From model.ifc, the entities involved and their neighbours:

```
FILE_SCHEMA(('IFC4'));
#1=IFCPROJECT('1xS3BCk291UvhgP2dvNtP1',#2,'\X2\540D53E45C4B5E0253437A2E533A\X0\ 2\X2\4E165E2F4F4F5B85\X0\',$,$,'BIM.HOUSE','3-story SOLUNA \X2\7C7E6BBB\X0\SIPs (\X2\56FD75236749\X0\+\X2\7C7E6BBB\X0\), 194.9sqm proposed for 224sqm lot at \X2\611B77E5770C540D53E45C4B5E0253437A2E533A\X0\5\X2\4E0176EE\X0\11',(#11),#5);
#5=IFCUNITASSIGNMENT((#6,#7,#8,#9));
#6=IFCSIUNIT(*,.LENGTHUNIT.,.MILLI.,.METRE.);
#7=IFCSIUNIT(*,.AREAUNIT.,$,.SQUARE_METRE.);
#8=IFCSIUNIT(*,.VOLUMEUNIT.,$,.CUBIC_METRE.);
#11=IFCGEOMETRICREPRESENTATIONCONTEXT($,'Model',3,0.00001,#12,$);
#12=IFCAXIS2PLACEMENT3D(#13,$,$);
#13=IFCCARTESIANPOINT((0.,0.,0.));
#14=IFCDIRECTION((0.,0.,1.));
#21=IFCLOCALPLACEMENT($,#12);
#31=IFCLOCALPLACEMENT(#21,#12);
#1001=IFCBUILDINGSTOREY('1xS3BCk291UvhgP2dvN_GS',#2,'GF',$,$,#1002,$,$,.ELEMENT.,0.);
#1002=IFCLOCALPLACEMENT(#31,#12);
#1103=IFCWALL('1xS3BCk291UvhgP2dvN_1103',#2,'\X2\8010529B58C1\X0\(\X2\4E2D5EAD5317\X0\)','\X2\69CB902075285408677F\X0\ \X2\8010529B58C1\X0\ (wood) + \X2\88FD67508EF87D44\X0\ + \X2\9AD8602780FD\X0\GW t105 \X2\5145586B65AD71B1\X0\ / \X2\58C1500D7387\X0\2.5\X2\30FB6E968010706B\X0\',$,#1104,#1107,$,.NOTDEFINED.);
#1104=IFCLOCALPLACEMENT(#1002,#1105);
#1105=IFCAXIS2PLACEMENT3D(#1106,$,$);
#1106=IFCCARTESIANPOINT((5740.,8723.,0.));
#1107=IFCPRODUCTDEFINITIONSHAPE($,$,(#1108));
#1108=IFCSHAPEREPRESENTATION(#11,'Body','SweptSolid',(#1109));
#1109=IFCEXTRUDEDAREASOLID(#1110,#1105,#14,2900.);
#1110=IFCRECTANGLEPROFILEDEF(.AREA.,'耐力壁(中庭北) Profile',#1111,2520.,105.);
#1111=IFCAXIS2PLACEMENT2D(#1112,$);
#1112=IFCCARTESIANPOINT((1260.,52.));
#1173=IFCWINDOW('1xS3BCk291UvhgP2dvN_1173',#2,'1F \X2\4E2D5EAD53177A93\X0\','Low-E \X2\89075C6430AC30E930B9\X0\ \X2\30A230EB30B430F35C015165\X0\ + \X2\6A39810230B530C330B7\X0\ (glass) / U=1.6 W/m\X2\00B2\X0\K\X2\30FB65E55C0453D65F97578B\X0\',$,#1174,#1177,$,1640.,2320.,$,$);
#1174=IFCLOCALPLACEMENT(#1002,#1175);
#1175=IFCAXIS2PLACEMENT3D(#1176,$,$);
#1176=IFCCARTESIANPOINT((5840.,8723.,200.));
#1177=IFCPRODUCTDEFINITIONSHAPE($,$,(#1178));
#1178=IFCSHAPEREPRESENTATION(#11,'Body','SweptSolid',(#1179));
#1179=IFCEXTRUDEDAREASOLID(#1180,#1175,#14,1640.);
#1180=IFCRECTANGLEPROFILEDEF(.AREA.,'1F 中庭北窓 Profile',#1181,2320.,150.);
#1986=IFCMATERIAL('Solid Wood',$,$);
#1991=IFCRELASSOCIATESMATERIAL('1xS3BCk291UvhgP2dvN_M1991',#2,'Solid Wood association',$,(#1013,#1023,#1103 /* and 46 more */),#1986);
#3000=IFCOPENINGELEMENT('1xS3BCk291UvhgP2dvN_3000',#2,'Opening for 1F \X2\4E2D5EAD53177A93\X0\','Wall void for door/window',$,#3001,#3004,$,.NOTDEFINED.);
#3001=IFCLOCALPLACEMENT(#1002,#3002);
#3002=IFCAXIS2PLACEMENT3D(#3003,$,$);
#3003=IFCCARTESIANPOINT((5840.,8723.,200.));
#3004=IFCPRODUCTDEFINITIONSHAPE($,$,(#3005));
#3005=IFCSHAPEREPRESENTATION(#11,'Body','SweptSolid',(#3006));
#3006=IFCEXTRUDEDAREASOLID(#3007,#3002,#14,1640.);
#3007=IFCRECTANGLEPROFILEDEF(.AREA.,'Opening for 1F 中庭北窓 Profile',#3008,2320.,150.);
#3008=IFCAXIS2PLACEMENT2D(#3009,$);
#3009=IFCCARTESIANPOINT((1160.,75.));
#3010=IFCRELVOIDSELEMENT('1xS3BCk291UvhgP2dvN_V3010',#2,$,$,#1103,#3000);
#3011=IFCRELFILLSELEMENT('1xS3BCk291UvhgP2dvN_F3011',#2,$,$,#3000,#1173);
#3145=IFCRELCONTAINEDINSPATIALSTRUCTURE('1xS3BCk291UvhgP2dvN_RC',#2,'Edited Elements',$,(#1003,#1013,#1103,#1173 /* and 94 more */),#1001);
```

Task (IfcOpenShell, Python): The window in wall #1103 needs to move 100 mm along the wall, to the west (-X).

```python
import ifcopenshell
import ifcopenshell.api.geometry
import ifcopenshell.util.placement
import ifcopenshell.util.unit

model = ifcopenshell.open("model.ifc")
unit_scale = ifcopenshell.util.unit.calculate_unit_scale(model)

window = model.by_guid("1xS3BCk291UvhgP2dvN_1173")
opening = window.FillsVoids[0].RelatingOpeningElement
wall = opening.VoidsElements[0].RelatingBuildingElement

wall_matrix = ifcopenshell.util.placement.get_local_placement(wall.ObjectPlacement)
shift = wall_matrix[:3, 0] * -0.1 / unit_scale
before = ifcopenshell.util.placement.get_local_placement(window.ObjectPlacement)[:3, 3].copy()

# The window is not placed relative to its opening, so move both.
for product in (opening, window):
    matrix = ifcopenshell.util.placement.get_local_placement(product.ObjectPlacement)
    matrix[:3, 3] += shift
    ifcopenshell.api.geometry.edit_object_placement(model, product=product, matrix=matrix, is_si=False)

after = ifcopenshell.util.placement.get_local_placement(window.ObjectPlacement)[:3, 3]
print("window moved by", (after - before).round(3) + 0.0)

model.write("model_edited.ifc")
```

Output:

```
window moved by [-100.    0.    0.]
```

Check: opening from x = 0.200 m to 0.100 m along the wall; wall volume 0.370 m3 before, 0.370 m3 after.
